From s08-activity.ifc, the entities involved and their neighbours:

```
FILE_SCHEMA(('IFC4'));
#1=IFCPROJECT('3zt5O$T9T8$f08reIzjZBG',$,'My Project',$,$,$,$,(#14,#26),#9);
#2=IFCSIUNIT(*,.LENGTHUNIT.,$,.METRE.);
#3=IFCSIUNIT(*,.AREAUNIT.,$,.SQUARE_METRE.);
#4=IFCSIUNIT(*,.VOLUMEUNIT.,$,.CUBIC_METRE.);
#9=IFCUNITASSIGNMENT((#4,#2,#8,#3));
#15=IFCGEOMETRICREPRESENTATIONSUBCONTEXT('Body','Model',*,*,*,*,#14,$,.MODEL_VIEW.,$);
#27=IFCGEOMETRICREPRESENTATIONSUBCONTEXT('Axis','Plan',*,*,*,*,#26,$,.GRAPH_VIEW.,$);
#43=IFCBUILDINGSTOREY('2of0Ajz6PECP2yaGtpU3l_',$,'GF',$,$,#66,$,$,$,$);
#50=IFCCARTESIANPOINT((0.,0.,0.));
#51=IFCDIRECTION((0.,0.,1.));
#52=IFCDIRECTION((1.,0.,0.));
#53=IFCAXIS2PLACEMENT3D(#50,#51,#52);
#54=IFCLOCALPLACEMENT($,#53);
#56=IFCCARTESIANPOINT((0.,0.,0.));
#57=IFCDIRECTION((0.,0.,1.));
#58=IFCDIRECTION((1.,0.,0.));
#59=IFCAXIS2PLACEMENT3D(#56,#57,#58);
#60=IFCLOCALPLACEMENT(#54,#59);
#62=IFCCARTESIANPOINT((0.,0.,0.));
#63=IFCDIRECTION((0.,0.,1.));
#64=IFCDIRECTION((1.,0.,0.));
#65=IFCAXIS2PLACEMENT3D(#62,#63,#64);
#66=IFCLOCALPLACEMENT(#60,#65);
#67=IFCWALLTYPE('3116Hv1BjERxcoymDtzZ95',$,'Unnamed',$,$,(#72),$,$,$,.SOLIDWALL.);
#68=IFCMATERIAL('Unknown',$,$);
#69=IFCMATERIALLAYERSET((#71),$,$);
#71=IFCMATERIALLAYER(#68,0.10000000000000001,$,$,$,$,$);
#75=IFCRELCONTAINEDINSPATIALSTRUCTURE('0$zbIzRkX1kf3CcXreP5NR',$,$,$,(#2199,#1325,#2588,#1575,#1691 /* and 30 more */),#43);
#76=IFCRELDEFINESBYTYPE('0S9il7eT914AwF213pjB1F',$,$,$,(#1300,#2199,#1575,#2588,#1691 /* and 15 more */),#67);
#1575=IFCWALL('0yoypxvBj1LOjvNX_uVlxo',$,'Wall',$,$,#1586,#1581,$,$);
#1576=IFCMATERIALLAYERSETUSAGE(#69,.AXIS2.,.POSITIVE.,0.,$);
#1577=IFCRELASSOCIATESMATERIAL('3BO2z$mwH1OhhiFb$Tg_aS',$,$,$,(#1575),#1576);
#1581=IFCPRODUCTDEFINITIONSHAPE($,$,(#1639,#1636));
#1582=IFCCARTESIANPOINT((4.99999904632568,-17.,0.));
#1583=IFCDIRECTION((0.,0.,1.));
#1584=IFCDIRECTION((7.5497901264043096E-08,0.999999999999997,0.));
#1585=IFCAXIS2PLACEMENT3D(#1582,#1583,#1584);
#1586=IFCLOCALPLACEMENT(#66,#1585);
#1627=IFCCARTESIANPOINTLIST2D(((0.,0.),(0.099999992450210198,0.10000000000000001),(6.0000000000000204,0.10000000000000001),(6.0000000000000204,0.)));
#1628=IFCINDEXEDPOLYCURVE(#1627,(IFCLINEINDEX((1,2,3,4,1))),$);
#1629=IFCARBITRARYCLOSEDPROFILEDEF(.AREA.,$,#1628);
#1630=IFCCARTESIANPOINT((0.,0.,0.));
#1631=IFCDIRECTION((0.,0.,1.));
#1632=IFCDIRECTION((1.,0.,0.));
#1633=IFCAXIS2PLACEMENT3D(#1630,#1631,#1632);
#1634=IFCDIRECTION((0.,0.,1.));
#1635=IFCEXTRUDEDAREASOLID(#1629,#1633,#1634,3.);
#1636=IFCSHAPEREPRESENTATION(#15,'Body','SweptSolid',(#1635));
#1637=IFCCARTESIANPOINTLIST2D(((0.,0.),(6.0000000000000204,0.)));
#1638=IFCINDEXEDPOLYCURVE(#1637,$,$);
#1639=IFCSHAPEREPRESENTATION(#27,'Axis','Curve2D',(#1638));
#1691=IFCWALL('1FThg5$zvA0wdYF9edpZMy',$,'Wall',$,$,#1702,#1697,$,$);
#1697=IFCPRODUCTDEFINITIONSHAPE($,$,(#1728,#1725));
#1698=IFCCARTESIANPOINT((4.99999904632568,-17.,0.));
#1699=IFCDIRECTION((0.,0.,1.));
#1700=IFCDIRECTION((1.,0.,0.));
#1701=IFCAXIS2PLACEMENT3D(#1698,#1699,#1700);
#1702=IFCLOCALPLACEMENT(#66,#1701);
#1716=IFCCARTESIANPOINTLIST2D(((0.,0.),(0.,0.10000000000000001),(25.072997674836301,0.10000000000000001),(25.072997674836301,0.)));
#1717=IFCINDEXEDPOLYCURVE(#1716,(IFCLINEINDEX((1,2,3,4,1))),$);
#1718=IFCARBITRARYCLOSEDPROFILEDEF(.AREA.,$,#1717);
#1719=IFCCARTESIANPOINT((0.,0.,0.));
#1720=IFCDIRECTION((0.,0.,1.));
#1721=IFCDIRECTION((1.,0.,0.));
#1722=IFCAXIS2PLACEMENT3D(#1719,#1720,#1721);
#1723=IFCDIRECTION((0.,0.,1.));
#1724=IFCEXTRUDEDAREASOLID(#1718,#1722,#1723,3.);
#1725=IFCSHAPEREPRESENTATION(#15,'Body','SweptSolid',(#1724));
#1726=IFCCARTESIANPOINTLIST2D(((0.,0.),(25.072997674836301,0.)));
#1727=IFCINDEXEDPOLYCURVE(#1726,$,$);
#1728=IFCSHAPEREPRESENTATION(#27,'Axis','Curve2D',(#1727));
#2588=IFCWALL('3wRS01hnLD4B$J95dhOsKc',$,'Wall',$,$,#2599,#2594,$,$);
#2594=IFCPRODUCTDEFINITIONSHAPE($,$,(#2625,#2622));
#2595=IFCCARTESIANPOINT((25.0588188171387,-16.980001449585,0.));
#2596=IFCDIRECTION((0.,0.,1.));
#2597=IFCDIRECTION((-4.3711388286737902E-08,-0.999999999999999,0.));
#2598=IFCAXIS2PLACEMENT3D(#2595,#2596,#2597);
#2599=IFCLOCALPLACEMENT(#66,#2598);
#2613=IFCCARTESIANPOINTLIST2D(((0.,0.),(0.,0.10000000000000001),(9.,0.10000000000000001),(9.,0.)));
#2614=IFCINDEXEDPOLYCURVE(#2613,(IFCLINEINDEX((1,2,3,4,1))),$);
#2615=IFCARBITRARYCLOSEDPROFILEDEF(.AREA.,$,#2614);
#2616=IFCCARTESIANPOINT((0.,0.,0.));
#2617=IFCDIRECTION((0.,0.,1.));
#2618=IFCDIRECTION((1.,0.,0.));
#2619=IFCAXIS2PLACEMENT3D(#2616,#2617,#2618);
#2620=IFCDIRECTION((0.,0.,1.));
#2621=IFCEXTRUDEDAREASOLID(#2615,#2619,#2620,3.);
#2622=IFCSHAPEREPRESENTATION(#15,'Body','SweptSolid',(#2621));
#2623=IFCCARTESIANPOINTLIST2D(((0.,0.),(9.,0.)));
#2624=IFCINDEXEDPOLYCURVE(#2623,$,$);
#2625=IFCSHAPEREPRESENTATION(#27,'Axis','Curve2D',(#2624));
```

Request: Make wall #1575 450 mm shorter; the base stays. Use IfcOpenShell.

```python
import ifcopenshell
import ifcopenshell.geom
import ifcopenshell.util.representation
import ifcopenshell.util.shape
import ifcopenshell.util.unit

model = ifcopenshell.open("s08-activity.ifc")
unit_scale = ifcopenshell.util.unit.calculate_unit_scale(model)
settings = ifcopenshell.geom.settings()


def volume(element):
    """Net volume in cubic metres, openings subtracted."""
    shape = ifcopenshell.geom.create_shape(settings, element)
    return ifcopenshell.util.shape.get_volume(shape.geometry)


wall = model.by_guid("0yoypxvBj1LOjvNX_uVlxo")
before = volume(wall)

body = ifcopenshell.util.representation.get_representation(wall, "Model", "Body")
solid = body.Items[0]
old_height = solid.Depth
solid.Depth -= 0.45 / unit_scale
after = volume(wall)

print(f"height {old_height:g} -> {solid.Depth:g}, volume {before:.3f} -> {after:.3f} m3")

model.write("s08-activity-out.ifc")
```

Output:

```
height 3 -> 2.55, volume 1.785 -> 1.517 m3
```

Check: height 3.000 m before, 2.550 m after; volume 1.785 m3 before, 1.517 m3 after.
